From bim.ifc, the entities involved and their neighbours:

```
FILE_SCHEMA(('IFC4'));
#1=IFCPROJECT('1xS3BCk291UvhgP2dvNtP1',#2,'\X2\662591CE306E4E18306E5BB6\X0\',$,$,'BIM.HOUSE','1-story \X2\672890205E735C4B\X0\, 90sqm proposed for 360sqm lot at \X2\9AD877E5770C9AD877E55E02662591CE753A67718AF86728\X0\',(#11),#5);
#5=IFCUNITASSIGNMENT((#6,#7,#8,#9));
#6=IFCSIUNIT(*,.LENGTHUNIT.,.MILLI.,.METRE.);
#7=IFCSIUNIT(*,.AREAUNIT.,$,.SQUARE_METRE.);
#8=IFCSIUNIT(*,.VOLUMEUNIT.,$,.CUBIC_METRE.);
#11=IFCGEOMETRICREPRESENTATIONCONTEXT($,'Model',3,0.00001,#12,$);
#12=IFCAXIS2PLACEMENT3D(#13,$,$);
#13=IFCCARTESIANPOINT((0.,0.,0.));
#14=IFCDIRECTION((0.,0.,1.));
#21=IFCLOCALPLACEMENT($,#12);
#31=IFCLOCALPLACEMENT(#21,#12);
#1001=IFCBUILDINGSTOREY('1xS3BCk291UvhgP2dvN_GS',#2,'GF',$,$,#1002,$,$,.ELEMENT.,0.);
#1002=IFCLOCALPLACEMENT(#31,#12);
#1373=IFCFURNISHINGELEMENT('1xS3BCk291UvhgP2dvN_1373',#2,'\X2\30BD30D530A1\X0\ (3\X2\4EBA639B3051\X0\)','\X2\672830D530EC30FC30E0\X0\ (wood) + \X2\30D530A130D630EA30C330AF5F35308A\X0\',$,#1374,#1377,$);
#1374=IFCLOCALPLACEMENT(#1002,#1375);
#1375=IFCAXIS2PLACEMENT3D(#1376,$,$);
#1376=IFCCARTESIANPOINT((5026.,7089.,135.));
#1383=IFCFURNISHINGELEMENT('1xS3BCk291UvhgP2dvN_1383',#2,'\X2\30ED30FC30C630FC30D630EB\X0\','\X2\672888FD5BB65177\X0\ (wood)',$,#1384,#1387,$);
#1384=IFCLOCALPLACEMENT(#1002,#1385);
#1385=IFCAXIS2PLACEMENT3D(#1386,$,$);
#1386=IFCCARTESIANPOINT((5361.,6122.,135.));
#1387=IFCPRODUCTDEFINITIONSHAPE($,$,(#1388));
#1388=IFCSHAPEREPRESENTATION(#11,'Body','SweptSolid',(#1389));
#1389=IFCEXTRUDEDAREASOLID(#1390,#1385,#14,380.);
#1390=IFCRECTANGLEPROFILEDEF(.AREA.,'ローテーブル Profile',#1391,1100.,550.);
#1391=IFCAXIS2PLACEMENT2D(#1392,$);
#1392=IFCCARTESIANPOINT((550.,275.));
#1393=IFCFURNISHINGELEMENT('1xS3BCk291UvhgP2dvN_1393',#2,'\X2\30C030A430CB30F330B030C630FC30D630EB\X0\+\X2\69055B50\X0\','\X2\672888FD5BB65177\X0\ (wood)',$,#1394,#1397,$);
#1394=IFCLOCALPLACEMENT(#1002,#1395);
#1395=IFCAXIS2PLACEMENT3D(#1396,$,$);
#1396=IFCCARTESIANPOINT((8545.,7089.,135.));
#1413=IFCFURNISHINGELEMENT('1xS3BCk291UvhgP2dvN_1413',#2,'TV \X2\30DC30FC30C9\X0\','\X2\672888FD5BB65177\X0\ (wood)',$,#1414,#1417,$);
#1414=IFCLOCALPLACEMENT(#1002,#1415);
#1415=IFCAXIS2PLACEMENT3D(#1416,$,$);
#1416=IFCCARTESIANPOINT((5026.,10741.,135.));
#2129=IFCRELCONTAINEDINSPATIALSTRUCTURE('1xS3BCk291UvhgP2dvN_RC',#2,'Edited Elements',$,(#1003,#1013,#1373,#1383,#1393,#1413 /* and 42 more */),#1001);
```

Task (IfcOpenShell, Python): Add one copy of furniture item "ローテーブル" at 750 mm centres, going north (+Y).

```python
import numpy as np
import ifcopenshell
import ifcopenshell.api.geometry
import ifcopenshell.api.root
import ifcopenshell.util.element
import ifcopenshell.util.placement
import ifcopenshell.util.unit

model = ifcopenshell.open("bim.ifc")
unit_scale = ifcopenshell.util.unit.calculate_unit_scale(model)


def reuse_history(source, copy):
    """copy_class also copies each property set's owner history, people and application; keep the originals."""
    for rel in copy.IsDefinedBy:
        if rel.is_a("IfcRelDefinesByProperties") and (history := rel.RelatingPropertyDefinition.OwnerHistory):
            rel.RelatingPropertyDefinition.OwnerHistory = source.OwnerHistory
            ifcopenshell.util.element.remove_deep2(model, history)


source = model.by_guid("1xS3BCk291UvhgP2dvN_1383")
base = ifcopenshell.util.placement.get_local_placement(source.ObjectPlacement)
step = np.array([0.0, 1.0, 0.0]) * 0.75 / unit_scale

for i in range(1, 2):
    copy = ifcopenshell.api.root.copy_class(model, product=source)
    copy.Representation = ifcopenshell.util.element.copy_deep(
        model, source.Representation, exclude=["IfcGeometricRepresentationContext", "IfcRepresentationMap"]
    )
    reuse_history(source, copy)
    matrix = base.copy()
    matrix[:3, 3] += i * step
    print("added at", matrix[:3, 3].round(3) + 0.0)
    ifcopenshell.api.geometry.edit_object_placement(model, product=copy, matrix=matrix, is_si=False)

model.write("bim-out.ifc")
```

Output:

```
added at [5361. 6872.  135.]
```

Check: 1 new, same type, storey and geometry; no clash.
